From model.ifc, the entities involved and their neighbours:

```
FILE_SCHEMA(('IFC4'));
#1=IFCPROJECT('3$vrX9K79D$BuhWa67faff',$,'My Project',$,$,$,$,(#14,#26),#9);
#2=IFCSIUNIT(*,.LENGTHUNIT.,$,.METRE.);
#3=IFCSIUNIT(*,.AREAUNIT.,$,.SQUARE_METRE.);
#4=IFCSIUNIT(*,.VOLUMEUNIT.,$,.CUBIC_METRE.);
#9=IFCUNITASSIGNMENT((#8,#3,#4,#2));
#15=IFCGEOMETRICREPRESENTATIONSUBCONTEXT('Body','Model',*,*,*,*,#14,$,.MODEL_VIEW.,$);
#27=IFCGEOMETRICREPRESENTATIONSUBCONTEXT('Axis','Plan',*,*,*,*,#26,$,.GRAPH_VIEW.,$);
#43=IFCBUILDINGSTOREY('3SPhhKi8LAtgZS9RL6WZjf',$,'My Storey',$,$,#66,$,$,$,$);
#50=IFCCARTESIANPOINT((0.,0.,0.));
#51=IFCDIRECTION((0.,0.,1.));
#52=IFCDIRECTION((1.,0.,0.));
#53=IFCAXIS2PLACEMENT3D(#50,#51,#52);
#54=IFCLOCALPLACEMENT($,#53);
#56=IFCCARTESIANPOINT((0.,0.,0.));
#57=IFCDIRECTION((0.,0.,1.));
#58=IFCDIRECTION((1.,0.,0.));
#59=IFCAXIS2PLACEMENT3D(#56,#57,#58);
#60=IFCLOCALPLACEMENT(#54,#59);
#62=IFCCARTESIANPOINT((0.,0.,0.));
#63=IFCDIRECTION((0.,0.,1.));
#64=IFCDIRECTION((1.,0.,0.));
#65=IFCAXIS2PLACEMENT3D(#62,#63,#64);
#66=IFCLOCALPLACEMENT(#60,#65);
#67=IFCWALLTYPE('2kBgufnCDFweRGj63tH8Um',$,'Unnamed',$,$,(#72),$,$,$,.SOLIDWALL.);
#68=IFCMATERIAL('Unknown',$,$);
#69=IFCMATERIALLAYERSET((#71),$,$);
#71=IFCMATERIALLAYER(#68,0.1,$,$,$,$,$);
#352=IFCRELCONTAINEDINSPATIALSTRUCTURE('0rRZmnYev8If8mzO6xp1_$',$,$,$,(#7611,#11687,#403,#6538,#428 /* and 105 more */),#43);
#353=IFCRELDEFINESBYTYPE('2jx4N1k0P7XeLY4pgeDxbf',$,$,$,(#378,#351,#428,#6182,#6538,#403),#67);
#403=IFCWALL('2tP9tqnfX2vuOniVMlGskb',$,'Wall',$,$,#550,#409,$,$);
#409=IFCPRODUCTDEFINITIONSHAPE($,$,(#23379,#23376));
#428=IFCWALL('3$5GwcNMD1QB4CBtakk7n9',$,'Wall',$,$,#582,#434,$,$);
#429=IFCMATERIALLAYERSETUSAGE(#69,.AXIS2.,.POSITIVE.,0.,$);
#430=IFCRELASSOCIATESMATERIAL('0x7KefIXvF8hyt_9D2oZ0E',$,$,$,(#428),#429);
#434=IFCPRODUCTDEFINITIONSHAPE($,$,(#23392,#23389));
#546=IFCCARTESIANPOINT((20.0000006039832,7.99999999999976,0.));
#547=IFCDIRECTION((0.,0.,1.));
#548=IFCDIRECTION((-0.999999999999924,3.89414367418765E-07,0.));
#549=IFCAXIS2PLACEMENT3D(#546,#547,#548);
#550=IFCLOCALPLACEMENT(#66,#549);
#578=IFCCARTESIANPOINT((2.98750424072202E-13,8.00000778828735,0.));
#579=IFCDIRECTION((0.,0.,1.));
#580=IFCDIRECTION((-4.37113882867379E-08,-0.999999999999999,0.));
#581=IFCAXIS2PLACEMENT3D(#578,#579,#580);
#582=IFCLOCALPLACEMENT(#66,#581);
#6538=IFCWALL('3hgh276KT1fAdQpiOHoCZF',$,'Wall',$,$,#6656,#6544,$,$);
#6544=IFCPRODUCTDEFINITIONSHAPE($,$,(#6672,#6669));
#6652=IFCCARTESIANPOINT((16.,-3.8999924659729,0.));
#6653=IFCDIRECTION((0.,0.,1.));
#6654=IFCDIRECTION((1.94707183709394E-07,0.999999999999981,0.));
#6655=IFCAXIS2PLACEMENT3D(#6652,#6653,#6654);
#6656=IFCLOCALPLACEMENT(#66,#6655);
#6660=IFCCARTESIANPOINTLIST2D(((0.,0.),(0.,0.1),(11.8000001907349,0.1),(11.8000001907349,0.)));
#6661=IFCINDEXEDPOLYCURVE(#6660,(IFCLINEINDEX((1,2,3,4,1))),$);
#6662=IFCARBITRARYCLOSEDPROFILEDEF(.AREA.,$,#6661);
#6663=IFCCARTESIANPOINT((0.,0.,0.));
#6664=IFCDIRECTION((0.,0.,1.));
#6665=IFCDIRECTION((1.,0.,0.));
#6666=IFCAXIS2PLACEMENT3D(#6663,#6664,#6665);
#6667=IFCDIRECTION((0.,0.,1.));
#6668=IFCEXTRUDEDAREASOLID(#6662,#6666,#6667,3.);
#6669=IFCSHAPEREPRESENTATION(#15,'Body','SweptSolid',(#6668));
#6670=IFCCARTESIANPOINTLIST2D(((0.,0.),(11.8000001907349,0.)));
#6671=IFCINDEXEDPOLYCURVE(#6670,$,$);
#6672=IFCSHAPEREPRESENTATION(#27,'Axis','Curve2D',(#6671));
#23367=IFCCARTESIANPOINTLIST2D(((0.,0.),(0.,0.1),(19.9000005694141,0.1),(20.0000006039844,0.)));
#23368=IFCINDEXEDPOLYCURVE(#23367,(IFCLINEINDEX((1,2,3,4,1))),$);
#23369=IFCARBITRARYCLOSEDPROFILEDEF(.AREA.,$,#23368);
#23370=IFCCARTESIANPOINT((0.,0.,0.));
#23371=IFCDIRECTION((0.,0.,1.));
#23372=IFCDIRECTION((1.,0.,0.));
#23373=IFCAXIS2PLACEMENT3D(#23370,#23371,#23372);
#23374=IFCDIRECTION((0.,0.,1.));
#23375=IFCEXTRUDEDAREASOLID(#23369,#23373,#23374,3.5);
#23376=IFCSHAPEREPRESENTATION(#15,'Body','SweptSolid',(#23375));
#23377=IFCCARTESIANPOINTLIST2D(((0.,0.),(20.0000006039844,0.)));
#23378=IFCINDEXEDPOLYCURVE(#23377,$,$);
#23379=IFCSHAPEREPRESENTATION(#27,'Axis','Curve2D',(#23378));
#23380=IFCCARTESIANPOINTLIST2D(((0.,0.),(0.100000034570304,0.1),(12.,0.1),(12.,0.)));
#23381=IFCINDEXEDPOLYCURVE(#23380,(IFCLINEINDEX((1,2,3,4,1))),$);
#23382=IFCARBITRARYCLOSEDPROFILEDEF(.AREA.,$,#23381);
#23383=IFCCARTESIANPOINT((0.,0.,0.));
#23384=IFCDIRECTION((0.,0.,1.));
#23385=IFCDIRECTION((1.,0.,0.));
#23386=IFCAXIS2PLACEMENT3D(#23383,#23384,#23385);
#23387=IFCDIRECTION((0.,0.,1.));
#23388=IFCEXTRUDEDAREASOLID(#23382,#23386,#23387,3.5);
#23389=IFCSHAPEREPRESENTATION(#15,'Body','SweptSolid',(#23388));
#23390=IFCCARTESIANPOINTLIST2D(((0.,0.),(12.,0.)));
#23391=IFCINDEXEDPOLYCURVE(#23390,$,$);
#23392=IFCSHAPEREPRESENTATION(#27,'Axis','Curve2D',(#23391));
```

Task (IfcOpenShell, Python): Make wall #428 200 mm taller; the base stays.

```python
import ifcopenshell
import ifcopenshell.geom
import ifcopenshell.util.representation
import ifcopenshell.util.shape
import ifcopenshell.util.unit

model = ifcopenshell.open("model.ifc")
unit_scale = ifcopenshell.util.unit.calculate_unit_scale(model)
settings = ifcopenshell.geom.settings()


def volume(element):
    """Net volume in cubic metres, openings subtracted."""
    shape = ifcopenshell.geom.create_shape(settings, element)
    return ifcopenshell.util.shape.get_volume(shape.geometry)


wall = model.by_guid("3$5GwcNMD1QB4CBtakk7n9")
before = volume(wall)

body = ifcopenshell.util.representation.get_representation(wall, "Model", "Body")
solid = body.Items[0]
old_height = solid.Depth
solid.Depth += 0.2 / unit_scale
after = volume(wall)

print(f"height {old_height:g} -> {solid.Depth:g}, volume {before:.3f} -> {after:.3f} m3")

model.write("model_edited.ifc")
```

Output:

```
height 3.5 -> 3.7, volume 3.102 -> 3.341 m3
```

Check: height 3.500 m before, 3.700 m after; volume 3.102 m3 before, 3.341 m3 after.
